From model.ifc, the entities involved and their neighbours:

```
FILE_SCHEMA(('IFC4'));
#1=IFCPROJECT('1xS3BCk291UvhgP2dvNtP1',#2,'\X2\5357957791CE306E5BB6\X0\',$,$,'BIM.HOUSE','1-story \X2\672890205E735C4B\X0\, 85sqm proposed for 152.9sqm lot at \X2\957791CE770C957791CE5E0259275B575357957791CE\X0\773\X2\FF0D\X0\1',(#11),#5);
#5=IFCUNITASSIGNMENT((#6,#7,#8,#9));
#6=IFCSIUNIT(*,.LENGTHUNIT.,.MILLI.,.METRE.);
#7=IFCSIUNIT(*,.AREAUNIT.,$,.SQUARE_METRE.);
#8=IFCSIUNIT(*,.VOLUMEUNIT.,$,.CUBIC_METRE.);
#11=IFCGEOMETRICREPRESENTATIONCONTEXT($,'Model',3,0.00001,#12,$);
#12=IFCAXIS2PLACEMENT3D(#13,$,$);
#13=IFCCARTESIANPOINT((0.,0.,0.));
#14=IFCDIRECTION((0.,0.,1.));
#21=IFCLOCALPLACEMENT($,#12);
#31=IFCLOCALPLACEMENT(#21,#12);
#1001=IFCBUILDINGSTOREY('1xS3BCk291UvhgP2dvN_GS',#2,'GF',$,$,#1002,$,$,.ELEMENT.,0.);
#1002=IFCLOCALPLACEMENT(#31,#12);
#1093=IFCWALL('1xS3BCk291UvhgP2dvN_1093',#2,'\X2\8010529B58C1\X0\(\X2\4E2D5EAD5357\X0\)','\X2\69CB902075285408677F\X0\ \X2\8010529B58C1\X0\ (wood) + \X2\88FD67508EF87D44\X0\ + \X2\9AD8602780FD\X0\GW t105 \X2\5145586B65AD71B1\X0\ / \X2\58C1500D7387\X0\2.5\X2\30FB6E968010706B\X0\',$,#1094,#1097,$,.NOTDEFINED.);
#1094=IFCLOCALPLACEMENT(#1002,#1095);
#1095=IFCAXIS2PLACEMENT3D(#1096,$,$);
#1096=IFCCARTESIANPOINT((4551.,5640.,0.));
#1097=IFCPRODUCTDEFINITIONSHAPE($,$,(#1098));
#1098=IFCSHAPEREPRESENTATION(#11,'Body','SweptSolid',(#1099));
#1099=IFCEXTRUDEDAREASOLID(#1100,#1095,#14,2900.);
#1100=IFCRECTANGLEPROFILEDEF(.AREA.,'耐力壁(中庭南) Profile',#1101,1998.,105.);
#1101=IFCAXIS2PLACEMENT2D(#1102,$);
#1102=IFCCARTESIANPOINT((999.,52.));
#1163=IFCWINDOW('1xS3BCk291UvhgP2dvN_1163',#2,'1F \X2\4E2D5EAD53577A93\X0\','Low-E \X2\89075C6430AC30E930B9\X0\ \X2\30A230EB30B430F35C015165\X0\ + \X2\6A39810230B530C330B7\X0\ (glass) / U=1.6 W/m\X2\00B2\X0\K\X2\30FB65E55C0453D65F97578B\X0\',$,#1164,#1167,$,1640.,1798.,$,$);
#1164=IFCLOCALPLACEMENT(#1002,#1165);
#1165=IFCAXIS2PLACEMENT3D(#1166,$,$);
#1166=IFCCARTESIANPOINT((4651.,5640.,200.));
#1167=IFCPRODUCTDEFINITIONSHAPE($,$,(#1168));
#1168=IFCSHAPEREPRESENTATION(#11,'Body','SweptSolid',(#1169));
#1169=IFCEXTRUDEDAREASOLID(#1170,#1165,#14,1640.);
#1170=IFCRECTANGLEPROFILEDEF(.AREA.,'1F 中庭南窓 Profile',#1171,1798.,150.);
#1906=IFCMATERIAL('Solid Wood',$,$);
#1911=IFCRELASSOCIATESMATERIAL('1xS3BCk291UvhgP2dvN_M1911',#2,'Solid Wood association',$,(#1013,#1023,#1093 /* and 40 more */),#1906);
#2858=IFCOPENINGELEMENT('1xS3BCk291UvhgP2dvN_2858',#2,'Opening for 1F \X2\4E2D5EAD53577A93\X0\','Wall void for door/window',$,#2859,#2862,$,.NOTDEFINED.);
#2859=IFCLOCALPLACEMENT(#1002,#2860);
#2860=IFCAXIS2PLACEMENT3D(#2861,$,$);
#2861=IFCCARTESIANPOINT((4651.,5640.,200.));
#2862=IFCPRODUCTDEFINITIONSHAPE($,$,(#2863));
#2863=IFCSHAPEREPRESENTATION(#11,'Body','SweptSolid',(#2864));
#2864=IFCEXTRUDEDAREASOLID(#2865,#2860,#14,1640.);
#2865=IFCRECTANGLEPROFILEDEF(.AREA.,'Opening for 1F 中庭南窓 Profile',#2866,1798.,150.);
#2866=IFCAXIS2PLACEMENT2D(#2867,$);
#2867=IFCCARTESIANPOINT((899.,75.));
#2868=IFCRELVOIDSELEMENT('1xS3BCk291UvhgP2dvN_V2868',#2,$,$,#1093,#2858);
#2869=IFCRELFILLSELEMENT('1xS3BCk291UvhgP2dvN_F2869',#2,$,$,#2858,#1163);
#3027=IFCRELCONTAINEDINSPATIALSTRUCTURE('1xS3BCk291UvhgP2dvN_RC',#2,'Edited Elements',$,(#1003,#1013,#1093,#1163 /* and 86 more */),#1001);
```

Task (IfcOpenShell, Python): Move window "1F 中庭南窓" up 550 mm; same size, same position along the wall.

```python
import numpy as np
import ifcopenshell
import ifcopenshell.api.geometry
import ifcopenshell.util.placement
import ifcopenshell.util.unit

model = ifcopenshell.open("model.ifc")
unit_scale = ifcopenshell.util.unit.calculate_unit_scale(model)

window = model.by_guid("1xS3BCk291UvhgP2dvN_1163")
opening = window.FillsVoids[0].RelatingOpeningElement
dz = 0.55 / unit_scale

shift = np.array([0.0, 0.0, dz])
# The window is not placed relative to its opening, so move both.
for product in (opening, window):
    matrix = ifcopenshell.util.placement.get_local_placement(product.ObjectPlacement)
    matrix[:3, 3] += shift
    ifcopenshell.api.geometry.edit_object_placement(model, product=product, matrix=matrix, is_si=False)

print(f"moved by {dz * unit_scale:+.3f} m")

model.write("model-out.ifc")
```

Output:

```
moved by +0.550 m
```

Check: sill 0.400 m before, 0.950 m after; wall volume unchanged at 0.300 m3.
